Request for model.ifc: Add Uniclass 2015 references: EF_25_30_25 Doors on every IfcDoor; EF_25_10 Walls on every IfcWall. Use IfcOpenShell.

First a look at what the model holds.

```python
import ifcopenshell

model = ifcopenshell.open("model.ifc")
print(model.schema)
print("classifications:", [c.Name for c in model.by_type("IfcClassification")])
for ifc_class in ("IfcDoor", "IfcRoof", "IfcStair", "IfcWall", "IfcWindow"):
    print(ifc_class, len(model.by_type(ifc_class)))
```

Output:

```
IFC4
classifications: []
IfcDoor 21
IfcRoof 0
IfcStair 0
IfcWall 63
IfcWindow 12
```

```python
import ifcopenshell
import ifcopenshell.api.classification

model = ifcopenshell.open("model.ifc")

system = ifcopenshell.api.classification.add_classification(model, classification="Uniclass 2015")

codes = {
    "IfcDoor": ("EF_25_30_25", "Doors"),
    "IfcWall": ("EF_25_10", "Walls"),
}
for ifc_class, (code, name) in codes.items():
    products = model.by_type(ifc_class)
    ifcopenshell.api.classification.add_reference(
        model, products=products, classification=system, identification=code, name=name
    )
    print(code, len(products))

model.write("model_rev.ifc")
```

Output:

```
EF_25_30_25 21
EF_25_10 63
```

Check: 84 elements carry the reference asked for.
